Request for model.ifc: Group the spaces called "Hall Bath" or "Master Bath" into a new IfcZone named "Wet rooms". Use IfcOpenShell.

First a look at what the model holds.

```python
import ifcopenshell

model = ifcopenshell.open("model.ifc")
print(model.schema)
seen = {}
for space in model.by_type("IfcSpace"):
    seen[space.LongName] = seen.get(space.LongName, 0) + 1
for name, count in sorted(seen.items(), key=str):
    print(count, "x", name)
print("zones:", [z.Name for z in model.by_type("IfcZone")][:20])
```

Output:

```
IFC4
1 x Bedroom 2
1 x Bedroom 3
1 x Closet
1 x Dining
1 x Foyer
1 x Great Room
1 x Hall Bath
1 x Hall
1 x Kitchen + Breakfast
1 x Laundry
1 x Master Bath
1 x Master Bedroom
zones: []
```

```python
import ifcopenshell
import ifcopenshell.api.group
import ifcopenshell.api.root

model = ifcopenshell.open("model.ifc")

names = {"Hall Bath", "Master Bath"}
spaces = [s for s in model.by_type("IfcSpace") if s.LongName in names]

zone = ifcopenshell.api.root.create_entity(model, ifc_class="IfcZone", name="Wet rooms")
ifcopenshell.api.group.assign_group(model, products=spaces, group=zone)
print(len(spaces), "spaces in", zone.Name)

model.write("model_rev.ifc")
```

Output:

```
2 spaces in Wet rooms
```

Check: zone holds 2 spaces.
